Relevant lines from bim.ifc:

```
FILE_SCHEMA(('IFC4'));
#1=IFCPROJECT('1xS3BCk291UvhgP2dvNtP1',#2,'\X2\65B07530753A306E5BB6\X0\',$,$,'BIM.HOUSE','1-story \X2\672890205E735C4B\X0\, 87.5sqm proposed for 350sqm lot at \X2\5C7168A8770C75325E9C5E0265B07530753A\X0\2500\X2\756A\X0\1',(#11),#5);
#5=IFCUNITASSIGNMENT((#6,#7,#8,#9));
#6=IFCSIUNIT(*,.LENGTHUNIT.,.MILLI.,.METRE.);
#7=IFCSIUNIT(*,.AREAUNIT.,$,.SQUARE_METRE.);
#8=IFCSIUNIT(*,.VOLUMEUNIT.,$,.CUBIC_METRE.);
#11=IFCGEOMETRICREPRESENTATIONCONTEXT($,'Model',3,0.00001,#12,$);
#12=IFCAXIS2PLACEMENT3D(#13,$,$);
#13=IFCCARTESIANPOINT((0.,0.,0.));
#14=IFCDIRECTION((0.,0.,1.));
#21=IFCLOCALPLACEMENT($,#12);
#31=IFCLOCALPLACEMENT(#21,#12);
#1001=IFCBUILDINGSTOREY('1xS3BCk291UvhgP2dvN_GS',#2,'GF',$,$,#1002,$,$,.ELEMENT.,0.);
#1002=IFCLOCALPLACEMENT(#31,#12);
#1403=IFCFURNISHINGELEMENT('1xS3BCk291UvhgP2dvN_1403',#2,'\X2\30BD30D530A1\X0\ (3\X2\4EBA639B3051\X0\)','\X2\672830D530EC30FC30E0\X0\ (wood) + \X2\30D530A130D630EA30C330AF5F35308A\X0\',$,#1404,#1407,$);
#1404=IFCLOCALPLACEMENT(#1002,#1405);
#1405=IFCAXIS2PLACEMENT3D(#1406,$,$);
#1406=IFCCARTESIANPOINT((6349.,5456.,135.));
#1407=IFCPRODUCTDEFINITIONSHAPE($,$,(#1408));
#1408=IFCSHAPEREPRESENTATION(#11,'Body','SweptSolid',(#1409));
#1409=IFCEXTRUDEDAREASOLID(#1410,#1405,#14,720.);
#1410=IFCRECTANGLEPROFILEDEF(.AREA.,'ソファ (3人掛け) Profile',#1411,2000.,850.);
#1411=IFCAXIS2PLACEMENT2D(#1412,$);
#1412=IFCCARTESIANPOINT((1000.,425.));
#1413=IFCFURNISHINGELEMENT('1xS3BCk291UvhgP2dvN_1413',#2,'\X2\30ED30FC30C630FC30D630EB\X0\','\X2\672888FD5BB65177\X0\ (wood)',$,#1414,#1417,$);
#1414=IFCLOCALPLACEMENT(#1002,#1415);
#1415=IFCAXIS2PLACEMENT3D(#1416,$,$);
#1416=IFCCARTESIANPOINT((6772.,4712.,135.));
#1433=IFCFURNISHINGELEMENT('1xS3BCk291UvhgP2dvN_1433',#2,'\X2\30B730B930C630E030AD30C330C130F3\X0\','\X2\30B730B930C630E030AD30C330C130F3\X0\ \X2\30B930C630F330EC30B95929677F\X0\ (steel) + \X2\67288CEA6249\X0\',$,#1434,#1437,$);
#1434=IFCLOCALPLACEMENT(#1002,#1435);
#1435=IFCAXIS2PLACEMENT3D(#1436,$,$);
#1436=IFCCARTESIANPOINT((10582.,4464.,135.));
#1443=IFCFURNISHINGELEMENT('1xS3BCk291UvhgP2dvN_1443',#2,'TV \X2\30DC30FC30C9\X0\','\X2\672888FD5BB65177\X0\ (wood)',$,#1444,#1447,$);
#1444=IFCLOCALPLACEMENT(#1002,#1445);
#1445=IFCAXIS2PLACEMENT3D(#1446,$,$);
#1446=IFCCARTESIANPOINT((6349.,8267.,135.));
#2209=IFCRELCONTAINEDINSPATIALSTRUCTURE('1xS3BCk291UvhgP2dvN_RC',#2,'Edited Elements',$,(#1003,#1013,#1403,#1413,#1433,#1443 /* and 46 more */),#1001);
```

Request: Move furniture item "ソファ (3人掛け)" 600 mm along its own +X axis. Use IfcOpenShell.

```python
import ifcopenshell
import ifcopenshell.api.geometry
import ifcopenshell.util.placement

model = ifcopenshell.open("bim.ifc")

item = model.by_id(1403)
matrix = ifcopenshell.util.placement.get_local_placement(item.ObjectPlacement)
matrix[:3, 3] += matrix[:3, 0] * 600.0
ifcopenshell.api.geometry.edit_object_placement(model, product=item, matrix=matrix, is_si=False)

print(ifcopenshell.util.placement.get_local_placement(item.ObjectPlacement).round(3) + 0.0)

model.write("bim_v2.ifc")
```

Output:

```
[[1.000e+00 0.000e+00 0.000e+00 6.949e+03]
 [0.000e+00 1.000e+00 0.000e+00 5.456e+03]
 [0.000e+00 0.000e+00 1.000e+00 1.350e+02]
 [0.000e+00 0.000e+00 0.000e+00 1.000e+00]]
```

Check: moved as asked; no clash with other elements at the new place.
